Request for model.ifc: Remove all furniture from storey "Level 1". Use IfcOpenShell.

First a look at what the model holds.

```python
import ifcopenshell
import ifcopenshell.util.element

model = ifcopenshell.open("model.ifc")
print(model.schema)
storey = next(s for s in model.by_type("IfcBuildingStorey") if s.Name == "Level 1")
furniture = [e for e in ifcopenshell.util.element.get_decomposition(storey) if e.is_a("IfcFurnishingElement")]
seen = {}
for e in furniture:
    element_type = ifcopenshell.util.element.get_type(e)
    name = element_type.Name if element_type not in (None, e) else None
    seen[name] = seen.get(name, 0) + 1
for name, count in sorted(seen.items(), key=str):
    print(count, "x", name)
```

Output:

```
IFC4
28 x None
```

```python
import ifcopenshell
import ifcopenshell.api.root
import ifcopenshell.util.element

model = ifcopenshell.open("model.ifc")

storey = next(s for s in model.by_type("IfcBuildingStorey") if s.Name == "Level 1")
furniture = [e for e in ifcopenshell.util.element.get_decomposition(storey) if e.is_a("IfcFurnishingElement")]

for e in furniture:
    ifcopenshell.api.root.remove_product(model, product=e)
print(len(furniture), "removed")

model.write("model_rev.ifc")
```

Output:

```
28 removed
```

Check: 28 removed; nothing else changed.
